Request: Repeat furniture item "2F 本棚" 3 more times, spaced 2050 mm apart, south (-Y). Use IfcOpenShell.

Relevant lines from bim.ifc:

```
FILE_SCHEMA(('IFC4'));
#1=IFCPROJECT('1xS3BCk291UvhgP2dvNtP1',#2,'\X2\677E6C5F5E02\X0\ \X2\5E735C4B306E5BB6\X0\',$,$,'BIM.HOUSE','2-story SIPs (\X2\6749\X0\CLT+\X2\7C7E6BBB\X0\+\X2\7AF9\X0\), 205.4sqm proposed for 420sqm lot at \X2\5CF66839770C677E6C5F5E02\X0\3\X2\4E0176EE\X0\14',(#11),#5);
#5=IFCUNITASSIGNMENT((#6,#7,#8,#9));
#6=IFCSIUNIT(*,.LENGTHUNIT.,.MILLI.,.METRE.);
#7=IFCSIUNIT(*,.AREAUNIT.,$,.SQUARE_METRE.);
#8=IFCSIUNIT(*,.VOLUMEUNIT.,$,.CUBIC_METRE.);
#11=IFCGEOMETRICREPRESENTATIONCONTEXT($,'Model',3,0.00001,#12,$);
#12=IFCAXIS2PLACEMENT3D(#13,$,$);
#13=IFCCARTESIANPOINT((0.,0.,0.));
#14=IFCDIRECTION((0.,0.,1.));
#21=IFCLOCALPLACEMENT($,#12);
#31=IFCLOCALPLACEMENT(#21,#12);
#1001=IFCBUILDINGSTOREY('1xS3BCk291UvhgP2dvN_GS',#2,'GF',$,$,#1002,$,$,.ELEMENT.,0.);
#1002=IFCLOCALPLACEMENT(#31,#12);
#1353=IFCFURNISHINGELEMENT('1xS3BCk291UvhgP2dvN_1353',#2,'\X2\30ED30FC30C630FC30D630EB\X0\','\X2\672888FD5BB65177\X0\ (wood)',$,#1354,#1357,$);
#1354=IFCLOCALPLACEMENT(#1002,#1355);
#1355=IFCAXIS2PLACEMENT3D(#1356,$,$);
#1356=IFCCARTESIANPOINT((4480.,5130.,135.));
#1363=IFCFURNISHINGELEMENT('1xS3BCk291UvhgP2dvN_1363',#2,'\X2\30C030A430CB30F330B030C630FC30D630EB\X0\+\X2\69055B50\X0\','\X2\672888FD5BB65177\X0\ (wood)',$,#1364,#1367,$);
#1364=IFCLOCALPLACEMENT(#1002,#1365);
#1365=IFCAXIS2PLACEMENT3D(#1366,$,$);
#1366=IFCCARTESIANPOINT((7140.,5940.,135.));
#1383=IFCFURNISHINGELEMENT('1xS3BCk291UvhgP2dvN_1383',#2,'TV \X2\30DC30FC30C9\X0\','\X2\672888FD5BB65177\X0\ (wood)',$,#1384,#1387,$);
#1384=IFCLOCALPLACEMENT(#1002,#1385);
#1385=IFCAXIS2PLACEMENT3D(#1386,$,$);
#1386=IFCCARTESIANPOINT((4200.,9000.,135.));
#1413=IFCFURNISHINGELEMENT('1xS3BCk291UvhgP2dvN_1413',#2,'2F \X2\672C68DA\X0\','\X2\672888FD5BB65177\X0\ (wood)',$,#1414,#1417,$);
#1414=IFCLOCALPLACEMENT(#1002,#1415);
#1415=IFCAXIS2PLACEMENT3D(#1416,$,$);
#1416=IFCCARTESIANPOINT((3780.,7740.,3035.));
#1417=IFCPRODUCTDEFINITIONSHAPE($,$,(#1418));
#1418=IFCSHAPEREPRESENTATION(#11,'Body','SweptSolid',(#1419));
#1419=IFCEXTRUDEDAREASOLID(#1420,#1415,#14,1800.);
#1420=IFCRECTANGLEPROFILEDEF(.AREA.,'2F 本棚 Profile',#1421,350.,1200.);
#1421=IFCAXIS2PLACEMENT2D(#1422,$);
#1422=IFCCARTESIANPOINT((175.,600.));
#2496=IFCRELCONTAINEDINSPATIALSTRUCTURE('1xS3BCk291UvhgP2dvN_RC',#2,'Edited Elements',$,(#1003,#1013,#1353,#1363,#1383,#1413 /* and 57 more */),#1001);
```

```python
import numpy as np
import ifcopenshell
import ifcopenshell.api.geometry
import ifcopenshell.api.root
import ifcopenshell.util.element
import ifcopenshell.util.placement
import ifcopenshell.util.unit

model = ifcopenshell.open("bim.ifc")
unit_scale = ifcopenshell.util.unit.calculate_unit_scale(model)


def reuse_history(source, copy):
    """copy_class also copies each property set's owner history, people and application; keep the originals."""
    for rel in copy.IsDefinedBy:
        if rel.is_a("IfcRelDefinesByProperties") and (history := rel.RelatingPropertyDefinition.OwnerHistory):
            rel.RelatingPropertyDefinition.OwnerHistory = source.OwnerHistory
            ifcopenshell.util.element.remove_deep2(model, history)


source = model.by_id(1413)
base = ifcopenshell.util.placement.get_local_placement(source.ObjectPlacement)
step = np.array([0.0, -1.0, 0.0]) * 2.05 / unit_scale

for i in range(1, 4):
    copy = ifcopenshell.api.root.copy_class(model, product=source)
    copy.Representation = ifcopenshell.util.element.copy_deep(
        model, source.Representation, exclude=["IfcGeometricRepresentationContext", "IfcRepresentationMap"]
    )
    reuse_history(source, copy)
    matrix = base.copy()
    matrix[:3, 3] += i * step
    print("added at", matrix[:3, 3].round(3) + 0.0)
    ifcopenshell.api.geometry.edit_object_placement(model, product=copy, matrix=matrix, is_si=False)

model.write("bim_rev.ifc")
```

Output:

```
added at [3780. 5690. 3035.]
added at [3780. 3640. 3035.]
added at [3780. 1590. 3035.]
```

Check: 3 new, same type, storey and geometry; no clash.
